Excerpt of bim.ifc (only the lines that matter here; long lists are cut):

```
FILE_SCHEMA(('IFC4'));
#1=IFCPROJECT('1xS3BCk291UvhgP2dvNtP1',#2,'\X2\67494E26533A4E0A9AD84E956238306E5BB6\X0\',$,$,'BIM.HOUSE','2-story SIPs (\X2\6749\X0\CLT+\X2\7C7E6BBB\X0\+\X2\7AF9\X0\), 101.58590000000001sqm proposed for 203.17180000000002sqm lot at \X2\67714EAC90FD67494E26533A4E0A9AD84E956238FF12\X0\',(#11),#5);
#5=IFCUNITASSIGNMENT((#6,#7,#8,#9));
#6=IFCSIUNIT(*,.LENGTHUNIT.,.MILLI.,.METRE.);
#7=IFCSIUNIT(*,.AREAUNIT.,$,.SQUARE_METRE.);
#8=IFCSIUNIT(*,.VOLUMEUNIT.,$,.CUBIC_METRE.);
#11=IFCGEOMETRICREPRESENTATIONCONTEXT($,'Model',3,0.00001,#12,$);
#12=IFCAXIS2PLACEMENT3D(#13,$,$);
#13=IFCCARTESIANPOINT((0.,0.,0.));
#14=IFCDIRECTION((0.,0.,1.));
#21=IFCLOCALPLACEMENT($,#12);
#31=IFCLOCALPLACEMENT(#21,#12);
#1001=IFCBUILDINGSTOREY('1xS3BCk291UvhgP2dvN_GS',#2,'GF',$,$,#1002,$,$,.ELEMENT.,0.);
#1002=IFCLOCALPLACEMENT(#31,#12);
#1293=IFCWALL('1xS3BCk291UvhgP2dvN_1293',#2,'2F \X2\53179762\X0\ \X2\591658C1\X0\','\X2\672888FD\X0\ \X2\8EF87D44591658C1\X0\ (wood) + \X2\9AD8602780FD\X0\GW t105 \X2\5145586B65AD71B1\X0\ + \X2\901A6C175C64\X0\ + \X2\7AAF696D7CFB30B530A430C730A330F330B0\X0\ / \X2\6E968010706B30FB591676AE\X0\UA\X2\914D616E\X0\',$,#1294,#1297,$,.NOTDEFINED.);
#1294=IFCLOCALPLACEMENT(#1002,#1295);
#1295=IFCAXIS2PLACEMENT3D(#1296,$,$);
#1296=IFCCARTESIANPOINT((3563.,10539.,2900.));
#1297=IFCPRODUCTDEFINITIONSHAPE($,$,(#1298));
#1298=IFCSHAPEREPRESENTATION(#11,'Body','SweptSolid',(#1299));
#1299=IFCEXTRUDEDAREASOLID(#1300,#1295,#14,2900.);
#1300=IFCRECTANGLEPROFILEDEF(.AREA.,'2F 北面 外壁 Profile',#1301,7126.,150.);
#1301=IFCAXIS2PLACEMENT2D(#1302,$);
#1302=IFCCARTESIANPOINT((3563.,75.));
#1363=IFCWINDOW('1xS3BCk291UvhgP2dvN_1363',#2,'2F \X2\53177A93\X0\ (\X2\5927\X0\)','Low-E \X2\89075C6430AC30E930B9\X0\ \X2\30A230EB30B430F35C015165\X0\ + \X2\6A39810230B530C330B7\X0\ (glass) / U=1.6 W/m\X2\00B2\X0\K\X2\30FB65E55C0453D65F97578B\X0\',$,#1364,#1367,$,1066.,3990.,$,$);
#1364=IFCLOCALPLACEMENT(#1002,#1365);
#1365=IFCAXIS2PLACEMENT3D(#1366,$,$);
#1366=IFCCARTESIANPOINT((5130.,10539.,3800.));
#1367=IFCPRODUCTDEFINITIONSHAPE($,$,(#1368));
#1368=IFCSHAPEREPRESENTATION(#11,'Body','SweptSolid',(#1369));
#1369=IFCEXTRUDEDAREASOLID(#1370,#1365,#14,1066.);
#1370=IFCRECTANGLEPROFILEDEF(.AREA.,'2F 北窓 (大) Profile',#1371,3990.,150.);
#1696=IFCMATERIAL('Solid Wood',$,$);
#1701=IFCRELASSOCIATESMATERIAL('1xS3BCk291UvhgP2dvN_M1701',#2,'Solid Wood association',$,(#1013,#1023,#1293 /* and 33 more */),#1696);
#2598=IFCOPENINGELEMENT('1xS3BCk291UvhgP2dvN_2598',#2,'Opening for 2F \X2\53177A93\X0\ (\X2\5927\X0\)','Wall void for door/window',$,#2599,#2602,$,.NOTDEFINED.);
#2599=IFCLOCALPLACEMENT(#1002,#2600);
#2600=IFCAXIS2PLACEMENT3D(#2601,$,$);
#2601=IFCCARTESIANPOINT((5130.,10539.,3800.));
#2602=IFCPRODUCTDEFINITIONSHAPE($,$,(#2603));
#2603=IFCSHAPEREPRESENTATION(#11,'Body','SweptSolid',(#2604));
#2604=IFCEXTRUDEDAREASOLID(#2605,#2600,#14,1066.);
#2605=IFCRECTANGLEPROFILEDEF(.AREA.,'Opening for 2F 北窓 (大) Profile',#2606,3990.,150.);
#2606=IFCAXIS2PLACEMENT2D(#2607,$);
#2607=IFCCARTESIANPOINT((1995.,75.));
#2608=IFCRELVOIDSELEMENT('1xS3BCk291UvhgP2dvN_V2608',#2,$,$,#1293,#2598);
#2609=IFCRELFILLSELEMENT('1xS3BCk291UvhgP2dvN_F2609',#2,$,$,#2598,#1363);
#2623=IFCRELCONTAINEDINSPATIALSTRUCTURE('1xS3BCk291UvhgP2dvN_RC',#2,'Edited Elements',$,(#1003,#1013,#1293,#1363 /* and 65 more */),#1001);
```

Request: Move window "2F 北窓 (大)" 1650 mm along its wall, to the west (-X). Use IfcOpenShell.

```python
import ifcopenshell
import ifcopenshell.api.geometry
import ifcopenshell.util.placement

model = ifcopenshell.open("bim.ifc")

window = model.by_guid("1xS3BCk291UvhgP2dvN_1363")
opening = window.FillsVoids[0].RelatingOpeningElement
wall = opening.VoidsElements[0].RelatingBuildingElement

wall_matrix = ifcopenshell.util.placement.get_local_placement(wall.ObjectPlacement)
shift = wall_matrix[:3, 0] * -1650.0
before = ifcopenshell.util.placement.get_local_placement(window.ObjectPlacement)[:3, 3].copy()

# The window is not placed relative to its opening, so move both.
for product in (opening, window):
    matrix = ifcopenshell.util.placement.get_local_placement(product.ObjectPlacement)
    matrix[:3, 3] += shift
    ifcopenshell.api.geometry.edit_object_placement(model, product=product, matrix=matrix, is_si=False)

after = ifcopenshell.util.placement.get_local_placement(window.ObjectPlacement)[:3, 3]
print("window moved by", (after - before).round(3) + 0.0)

model.write("bim_edited.ifc")
```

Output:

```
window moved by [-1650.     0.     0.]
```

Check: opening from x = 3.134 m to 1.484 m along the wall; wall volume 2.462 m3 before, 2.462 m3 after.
